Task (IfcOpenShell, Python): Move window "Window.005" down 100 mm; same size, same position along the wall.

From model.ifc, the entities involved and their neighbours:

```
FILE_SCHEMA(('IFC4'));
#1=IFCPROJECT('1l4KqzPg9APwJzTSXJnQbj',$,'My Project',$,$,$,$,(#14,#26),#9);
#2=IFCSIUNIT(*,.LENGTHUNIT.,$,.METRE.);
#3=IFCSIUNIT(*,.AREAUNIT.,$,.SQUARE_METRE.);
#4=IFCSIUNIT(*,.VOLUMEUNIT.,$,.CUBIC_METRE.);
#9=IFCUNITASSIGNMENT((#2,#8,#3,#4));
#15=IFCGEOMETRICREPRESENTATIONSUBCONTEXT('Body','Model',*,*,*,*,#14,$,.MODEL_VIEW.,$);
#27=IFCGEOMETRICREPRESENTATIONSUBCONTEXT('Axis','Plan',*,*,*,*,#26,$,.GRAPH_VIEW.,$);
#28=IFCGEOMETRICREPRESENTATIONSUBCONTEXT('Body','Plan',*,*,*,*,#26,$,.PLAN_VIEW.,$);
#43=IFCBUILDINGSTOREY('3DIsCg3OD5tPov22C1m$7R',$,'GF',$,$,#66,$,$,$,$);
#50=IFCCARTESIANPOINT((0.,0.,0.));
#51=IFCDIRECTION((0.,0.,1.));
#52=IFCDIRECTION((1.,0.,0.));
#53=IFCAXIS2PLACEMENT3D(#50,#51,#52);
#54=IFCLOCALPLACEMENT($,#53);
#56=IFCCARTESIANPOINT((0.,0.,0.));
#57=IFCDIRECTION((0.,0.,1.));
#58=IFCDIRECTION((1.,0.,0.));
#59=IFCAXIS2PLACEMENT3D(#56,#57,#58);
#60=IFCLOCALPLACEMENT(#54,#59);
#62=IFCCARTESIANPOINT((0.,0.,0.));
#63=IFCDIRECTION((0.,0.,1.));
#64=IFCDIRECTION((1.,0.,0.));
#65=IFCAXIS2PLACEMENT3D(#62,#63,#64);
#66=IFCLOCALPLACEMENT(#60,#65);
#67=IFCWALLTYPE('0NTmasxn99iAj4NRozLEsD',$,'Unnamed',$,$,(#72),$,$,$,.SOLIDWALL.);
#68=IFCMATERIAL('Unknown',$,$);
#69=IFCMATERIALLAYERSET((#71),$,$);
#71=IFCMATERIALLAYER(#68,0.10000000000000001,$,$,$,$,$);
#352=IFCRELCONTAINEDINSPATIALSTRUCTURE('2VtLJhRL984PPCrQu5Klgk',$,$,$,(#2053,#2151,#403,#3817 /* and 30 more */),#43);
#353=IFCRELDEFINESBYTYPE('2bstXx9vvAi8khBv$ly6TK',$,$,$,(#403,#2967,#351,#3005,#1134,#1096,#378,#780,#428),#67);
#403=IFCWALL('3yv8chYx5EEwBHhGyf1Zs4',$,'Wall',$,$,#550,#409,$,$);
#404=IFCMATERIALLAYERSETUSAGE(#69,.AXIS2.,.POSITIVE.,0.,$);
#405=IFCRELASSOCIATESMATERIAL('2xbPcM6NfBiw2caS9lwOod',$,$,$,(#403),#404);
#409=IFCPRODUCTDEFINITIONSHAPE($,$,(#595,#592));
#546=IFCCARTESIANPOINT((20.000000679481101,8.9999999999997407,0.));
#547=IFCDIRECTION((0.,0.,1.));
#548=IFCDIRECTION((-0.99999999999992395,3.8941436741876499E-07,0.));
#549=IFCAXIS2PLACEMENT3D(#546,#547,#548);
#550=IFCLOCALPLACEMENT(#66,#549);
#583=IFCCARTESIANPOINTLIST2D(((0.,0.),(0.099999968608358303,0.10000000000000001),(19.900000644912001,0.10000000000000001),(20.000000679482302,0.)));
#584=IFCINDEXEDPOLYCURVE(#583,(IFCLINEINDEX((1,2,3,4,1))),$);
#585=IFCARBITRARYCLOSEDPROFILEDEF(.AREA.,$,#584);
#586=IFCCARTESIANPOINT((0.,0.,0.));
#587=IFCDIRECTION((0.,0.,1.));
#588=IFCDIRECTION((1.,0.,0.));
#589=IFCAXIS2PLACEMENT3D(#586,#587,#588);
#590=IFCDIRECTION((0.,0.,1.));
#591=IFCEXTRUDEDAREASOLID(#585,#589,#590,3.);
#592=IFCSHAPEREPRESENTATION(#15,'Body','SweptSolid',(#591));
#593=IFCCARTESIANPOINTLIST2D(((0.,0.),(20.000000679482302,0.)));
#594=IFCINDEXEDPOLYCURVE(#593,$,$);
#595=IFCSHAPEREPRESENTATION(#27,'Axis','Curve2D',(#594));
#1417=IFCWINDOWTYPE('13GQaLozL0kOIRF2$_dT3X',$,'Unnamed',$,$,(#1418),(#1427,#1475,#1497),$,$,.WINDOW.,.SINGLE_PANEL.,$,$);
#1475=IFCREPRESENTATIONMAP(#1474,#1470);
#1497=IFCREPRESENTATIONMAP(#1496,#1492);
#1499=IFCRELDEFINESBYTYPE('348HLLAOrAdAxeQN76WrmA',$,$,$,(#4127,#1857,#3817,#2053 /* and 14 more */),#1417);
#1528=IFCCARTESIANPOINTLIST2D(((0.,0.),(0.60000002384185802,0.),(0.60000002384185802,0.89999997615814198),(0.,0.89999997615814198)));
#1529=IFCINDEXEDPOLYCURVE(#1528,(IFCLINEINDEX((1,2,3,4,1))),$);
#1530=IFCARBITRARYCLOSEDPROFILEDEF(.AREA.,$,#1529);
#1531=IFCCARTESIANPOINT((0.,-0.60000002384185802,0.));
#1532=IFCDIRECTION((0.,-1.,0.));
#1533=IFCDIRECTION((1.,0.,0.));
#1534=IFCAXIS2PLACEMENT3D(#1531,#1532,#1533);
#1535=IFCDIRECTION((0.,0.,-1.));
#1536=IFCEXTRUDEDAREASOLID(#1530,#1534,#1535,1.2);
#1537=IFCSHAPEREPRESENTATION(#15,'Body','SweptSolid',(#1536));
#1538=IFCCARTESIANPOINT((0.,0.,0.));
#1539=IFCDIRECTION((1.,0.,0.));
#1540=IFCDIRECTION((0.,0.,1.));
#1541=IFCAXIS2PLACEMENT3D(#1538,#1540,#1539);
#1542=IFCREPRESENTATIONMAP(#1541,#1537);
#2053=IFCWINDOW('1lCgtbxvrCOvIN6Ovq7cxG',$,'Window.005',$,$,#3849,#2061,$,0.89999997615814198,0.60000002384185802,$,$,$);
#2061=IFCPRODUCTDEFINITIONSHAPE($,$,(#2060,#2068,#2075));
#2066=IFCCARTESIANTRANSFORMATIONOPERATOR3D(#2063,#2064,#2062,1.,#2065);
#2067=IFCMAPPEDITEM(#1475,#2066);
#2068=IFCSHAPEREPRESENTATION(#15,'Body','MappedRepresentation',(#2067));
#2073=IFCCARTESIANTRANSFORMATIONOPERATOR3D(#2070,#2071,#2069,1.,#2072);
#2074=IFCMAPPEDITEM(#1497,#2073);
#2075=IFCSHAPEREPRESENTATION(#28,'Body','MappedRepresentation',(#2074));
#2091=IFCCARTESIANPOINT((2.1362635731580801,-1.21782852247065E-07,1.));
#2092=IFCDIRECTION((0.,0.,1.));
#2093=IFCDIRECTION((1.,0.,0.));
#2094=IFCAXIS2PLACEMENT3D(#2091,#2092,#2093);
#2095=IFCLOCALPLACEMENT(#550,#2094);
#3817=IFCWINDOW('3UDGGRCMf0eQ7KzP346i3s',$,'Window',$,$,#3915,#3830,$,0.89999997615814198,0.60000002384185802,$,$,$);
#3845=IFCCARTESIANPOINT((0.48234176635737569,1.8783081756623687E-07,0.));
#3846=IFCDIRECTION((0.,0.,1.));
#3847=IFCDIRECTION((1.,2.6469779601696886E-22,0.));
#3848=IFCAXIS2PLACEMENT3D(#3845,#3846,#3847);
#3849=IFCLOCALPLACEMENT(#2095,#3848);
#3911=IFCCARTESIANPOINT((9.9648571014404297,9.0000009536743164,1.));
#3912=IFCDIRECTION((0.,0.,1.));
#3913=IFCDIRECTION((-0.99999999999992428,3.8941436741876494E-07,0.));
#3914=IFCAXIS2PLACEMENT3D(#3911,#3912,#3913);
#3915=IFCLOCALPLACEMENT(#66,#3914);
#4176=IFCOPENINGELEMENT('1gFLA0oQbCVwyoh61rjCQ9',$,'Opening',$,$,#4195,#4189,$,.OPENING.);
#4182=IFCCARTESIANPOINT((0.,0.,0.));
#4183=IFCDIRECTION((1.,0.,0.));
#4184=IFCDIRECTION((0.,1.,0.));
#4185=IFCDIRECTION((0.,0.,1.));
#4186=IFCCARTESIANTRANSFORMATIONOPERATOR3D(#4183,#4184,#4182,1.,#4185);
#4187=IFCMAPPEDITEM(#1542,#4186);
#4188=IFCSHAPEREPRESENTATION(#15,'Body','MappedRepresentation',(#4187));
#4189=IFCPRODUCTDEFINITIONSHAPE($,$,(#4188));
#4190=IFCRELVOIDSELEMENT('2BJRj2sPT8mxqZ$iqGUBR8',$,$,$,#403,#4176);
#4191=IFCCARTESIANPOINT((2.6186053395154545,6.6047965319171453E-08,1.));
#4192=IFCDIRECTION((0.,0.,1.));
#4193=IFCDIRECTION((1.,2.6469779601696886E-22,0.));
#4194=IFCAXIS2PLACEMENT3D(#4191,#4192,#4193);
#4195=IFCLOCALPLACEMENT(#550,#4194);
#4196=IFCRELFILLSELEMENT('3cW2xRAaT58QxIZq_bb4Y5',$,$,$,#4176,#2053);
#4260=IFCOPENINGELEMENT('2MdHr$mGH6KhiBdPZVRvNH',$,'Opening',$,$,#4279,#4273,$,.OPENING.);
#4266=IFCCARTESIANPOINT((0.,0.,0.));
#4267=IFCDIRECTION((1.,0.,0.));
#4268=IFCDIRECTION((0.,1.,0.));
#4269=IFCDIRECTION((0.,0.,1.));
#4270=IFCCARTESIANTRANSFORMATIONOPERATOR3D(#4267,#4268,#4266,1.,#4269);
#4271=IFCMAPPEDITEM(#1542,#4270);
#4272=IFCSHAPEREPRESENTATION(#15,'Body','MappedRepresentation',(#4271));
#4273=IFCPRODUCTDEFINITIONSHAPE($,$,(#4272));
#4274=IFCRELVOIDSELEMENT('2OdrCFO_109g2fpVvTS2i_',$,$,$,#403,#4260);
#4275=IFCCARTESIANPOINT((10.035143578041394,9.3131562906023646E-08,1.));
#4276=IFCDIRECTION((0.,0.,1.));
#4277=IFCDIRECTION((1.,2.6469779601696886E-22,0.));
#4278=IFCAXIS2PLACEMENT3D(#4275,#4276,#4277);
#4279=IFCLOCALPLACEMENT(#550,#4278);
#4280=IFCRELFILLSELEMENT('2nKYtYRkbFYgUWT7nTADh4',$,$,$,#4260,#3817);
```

```python
import numpy as np
import ifcopenshell
import ifcopenshell.api.geometry
import ifcopenshell.util.placement
import ifcopenshell.util.unit

model = ifcopenshell.open("model.ifc")
unit_scale = ifcopenshell.util.unit.calculate_unit_scale(model)

window = model.by_guid("1lCgtbxvrCOvIN6Ovq7cxG")
opening = window.FillsVoids[0].RelatingOpeningElement
dz = -0.1

shift = np.array([0.0, 0.0, dz])
# The window is not placed relative to its opening, so move both.
for product in (opening, window):
    matrix = ifcopenshell.util.placement.get_local_placement(product.ObjectPlacement)
    matrix[:3, 3] += shift
    ifcopenshell.api.geometry.edit_object_placement(model, product=product, matrix=matrix, is_si=False)

print(f"moved by {dz * unit_scale:+.3f} m")

model.write("model_rev.ifc")
```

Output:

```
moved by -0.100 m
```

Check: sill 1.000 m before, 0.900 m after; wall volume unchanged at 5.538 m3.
